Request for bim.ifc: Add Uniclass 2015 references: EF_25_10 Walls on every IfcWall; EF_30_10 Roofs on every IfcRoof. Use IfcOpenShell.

First a look at what the model holds.

```python
import ifcopenshell

model = ifcopenshell.open("bim.ifc")
print(model.schema)
print("classifications:", [c.Name for c in model.by_type("IfcClassification")])
for ifc_class in ("IfcDoor", "IfcRoof", "IfcStair", "IfcWall", "IfcWindow"):
    print(ifc_class, len(model.by_type(ifc_class)))
```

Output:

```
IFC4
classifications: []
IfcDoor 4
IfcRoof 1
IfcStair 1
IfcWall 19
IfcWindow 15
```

```python
import ifcopenshell
import ifcopenshell.api.classification

model = ifcopenshell.open("bim.ifc")

system = ifcopenshell.api.classification.add_classification(model, classification="Uniclass 2015")

codes = {
    "IfcWall": ("EF_25_10", "Walls"),
    "IfcRoof": ("EF_30_10", "Roofs"),
}
for ifc_class, (code, name) in codes.items():
    products = model.by_type(ifc_class)
    ifcopenshell.api.classification.add_reference(
        model, products=products, classification=system, identification=code, name=name
    )
    print(code, len(products))

model.write("bim_rev.ifc")
```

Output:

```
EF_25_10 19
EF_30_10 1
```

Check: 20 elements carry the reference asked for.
